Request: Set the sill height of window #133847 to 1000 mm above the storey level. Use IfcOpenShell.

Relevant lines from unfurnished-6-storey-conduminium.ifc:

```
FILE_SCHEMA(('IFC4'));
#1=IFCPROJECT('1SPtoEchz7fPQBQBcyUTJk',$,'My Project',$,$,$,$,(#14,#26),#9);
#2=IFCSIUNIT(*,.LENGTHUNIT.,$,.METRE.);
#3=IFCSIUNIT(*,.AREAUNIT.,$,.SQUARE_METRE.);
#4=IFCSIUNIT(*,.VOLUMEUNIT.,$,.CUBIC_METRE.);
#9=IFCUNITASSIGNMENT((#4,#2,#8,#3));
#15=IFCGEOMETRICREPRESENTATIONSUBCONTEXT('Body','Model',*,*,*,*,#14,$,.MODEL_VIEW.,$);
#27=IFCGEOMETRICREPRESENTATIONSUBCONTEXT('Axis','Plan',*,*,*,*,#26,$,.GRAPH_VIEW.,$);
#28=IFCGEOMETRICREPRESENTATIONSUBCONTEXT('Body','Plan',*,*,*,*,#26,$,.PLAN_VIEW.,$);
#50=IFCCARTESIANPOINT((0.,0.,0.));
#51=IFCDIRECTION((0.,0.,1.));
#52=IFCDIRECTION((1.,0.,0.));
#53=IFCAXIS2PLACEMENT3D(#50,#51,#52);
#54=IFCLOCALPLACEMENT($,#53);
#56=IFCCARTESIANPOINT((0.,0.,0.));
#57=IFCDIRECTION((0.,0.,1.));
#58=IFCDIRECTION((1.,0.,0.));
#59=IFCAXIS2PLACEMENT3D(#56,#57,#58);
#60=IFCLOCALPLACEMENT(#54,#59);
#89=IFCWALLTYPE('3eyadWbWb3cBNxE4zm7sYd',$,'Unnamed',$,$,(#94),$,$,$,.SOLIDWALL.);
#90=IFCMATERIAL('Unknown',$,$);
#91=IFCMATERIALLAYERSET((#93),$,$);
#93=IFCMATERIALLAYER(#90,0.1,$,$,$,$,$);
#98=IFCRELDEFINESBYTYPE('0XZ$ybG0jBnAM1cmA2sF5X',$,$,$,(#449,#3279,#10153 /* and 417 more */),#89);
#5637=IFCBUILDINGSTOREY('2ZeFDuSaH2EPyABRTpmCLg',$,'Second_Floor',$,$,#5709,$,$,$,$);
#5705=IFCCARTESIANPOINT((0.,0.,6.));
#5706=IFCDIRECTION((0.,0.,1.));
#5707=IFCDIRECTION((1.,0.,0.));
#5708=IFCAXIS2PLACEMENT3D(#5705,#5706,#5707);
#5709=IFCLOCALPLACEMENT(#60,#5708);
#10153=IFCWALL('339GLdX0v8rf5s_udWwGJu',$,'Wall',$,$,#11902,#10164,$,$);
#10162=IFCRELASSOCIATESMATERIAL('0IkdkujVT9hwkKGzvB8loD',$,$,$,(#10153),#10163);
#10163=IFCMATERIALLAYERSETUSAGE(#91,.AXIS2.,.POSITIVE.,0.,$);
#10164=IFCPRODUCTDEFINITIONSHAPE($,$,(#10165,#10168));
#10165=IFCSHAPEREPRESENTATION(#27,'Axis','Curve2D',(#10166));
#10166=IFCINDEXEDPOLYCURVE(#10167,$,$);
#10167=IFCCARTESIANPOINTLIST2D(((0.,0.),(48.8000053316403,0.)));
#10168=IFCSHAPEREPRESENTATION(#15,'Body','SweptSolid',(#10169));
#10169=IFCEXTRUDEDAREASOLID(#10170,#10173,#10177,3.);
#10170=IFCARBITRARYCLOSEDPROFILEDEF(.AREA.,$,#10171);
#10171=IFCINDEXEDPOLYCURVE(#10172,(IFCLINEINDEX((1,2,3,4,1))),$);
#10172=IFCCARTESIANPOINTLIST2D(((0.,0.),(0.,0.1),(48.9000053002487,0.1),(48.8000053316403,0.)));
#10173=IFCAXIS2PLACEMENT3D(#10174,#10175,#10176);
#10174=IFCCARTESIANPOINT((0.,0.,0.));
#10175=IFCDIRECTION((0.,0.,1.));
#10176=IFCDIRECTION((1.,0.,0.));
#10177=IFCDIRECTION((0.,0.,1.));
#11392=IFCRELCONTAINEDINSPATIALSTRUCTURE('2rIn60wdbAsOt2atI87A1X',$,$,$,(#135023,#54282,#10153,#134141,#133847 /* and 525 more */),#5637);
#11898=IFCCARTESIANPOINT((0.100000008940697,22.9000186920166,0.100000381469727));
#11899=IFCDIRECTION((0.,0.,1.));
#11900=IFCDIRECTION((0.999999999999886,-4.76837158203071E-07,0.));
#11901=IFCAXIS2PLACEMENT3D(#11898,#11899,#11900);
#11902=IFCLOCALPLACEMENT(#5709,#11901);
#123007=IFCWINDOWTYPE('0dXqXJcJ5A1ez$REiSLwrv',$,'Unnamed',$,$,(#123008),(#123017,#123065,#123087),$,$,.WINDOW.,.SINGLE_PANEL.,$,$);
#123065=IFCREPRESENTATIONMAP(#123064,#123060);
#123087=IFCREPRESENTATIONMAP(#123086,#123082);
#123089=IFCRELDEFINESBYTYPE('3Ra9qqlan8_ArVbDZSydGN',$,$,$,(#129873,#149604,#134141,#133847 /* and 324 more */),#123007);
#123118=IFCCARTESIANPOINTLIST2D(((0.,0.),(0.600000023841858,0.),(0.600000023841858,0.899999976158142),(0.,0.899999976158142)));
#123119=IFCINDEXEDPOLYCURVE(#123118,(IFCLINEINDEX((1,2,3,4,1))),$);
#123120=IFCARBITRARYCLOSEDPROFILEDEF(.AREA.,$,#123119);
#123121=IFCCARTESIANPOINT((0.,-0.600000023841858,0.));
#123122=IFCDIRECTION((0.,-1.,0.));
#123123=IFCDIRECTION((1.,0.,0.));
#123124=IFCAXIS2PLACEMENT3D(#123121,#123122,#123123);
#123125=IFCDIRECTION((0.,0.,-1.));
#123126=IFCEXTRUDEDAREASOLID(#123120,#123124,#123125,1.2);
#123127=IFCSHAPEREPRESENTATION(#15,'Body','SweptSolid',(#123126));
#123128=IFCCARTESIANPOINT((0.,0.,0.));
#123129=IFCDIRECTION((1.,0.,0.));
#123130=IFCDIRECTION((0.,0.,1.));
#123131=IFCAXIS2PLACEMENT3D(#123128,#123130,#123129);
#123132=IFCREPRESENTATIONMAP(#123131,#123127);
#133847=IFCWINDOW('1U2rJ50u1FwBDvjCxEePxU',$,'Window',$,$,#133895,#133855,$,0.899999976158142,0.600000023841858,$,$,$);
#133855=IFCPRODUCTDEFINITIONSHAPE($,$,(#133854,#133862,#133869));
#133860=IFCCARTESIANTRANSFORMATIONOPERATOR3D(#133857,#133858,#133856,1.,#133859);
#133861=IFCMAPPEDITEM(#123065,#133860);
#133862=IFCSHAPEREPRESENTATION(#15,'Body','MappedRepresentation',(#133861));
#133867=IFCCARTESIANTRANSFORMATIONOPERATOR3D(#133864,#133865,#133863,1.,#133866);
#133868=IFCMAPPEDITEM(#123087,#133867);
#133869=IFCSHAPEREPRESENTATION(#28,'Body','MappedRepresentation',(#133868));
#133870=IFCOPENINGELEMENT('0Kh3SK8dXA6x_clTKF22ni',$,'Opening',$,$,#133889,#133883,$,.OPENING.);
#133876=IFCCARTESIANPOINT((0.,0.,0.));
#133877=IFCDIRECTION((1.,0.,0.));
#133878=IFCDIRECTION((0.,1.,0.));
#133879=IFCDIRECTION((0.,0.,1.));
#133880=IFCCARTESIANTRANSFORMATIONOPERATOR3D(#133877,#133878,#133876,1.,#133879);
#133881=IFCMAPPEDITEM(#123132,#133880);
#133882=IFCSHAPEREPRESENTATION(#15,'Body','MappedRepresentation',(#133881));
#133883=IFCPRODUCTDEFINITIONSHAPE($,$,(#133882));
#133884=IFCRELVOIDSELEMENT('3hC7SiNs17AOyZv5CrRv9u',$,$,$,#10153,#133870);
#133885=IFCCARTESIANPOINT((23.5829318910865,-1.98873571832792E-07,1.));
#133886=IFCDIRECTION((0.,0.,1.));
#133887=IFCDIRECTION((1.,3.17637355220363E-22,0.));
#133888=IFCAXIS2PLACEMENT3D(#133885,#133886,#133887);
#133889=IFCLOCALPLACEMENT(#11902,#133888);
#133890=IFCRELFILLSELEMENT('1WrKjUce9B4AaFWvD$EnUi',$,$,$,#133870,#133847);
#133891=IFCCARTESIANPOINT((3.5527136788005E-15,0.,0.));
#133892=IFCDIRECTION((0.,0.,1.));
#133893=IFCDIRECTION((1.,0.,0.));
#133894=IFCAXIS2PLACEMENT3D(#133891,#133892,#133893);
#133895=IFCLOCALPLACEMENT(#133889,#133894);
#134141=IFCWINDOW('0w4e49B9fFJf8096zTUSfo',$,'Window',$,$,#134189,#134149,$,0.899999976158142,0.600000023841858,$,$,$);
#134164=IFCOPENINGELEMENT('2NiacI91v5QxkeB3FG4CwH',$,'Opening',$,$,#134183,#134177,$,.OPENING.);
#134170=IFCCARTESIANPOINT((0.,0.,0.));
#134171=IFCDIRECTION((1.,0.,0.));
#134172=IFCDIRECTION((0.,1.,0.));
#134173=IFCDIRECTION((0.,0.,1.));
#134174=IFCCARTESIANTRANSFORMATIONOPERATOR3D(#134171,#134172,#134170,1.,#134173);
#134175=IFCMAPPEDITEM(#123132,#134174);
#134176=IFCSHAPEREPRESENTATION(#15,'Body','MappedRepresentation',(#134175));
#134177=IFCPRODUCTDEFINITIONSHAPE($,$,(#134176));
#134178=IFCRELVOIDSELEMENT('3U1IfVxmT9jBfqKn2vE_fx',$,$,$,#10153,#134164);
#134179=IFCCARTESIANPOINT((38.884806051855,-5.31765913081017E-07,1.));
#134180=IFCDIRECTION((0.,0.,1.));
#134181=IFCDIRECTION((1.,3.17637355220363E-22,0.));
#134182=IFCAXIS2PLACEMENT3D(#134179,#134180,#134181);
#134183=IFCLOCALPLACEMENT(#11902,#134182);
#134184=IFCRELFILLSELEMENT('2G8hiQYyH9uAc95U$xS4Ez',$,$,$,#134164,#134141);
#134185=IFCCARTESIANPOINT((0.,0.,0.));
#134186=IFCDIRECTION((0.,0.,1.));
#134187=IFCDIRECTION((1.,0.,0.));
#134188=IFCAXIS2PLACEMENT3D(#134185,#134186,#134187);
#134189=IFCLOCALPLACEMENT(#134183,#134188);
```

```python
import numpy as np
import ifcopenshell
import ifcopenshell.api.geometry
import ifcopenshell.geom
import ifcopenshell.util.element
import ifcopenshell.util.placement
import ifcopenshell.util.shape
import ifcopenshell.util.unit

model = ifcopenshell.open("unfurnished-6-storey-conduminium.ifc")
unit_scale = ifcopenshell.util.unit.calculate_unit_scale(model)

window = model.by_guid("1U2rJ50u1FwBDvjCxEePxU")
opening = window.FillsVoids[0].RelatingOpeningElement
storey = ifcopenshell.util.element.get_container(window, ifc_class="IfcBuildingStorey")
level = ifcopenshell.util.placement.get_local_placement(storey.ObjectPlacement)[2, 3]

# The opening's origin need not be at the sill, so measure its lowest point.
shape = ifcopenshell.geom.create_shape(ifcopenshell.geom.settings(), opening)
bottom = ifcopenshell.util.shape.get_shape_bottom_elevation(shape, shape.geometry) / unit_scale
dz = level + 1.0 - bottom

shift = np.array([0.0, 0.0, dz])
# The window is placed relative to its opening, so it follows when the opening moves.
matrix = ifcopenshell.util.placement.get_local_placement(opening.ObjectPlacement)
matrix[:3, 3] += shift
ifcopenshell.api.geometry.edit_object_placement(
    model, product=opening, matrix=matrix, is_si=False, should_transform_children=True
)

print(f"moved by {dz * unit_scale:+.3f} m")

model.write("unfurnished-6-storey-conduminium_updated.ifc")
```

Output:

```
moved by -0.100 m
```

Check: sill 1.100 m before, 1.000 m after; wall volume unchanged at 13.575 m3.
